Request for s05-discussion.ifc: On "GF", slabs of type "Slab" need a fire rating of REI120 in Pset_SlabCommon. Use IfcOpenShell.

First a look at what the model holds.

```python
import ifcopenshell
import ifcopenshell.util.element

model = ifcopenshell.open("s05-discussion.ifc")
print(model.schema)
storey = next(s for s in model.by_type("IfcBuildingStorey") if s.Name == "GF")
slabs = [e for e in ifcopenshell.util.element.get_decomposition(storey) if e.is_a("IfcSlab")]
seen = {}
for e in slabs:
    element_type = ifcopenshell.util.element.get_type(e)
    key = (element_type.Name if element_type != e and element_type else None, ifcopenshell.util.element.get_pset(e, "Pset_SlabCommon", "FireRating"))
    seen[key] = seen.get(key, 0) + 1
for (name, value), count in sorted(seen.items(), key=str):
    print(count, "x", name, "|", value)
```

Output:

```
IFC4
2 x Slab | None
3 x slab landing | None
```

```python
import ifcopenshell
import ifcopenshell.api.pset
import ifcopenshell.util.element

model = ifcopenshell.open("s05-discussion.ifc")

storey = next(s for s in model.by_type("IfcBuildingStorey") if s.Name == "GF")
slabs = [e for e in ifcopenshell.util.element.get_decomposition(storey) if e.is_a("IfcSlab")]

count = 0
for e in slabs:
    element_type = ifcopenshell.util.element.get_type(e)
    if element_type in (None, e) or element_type.Name != "Slab":
        continue
    # add_pset returns the element's existing set when there is one.
    pset = ifcopenshell.api.pset.add_pset(model, product=e, name="Pset_SlabCommon")
    ifcopenshell.api.pset.edit_pset(model, pset=pset, properties={"FireRating": "REI120"})
    count += 1

print(count, "slabs updated")

model.write("s05-discussion-out.ifc")
```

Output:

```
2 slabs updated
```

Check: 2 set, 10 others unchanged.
